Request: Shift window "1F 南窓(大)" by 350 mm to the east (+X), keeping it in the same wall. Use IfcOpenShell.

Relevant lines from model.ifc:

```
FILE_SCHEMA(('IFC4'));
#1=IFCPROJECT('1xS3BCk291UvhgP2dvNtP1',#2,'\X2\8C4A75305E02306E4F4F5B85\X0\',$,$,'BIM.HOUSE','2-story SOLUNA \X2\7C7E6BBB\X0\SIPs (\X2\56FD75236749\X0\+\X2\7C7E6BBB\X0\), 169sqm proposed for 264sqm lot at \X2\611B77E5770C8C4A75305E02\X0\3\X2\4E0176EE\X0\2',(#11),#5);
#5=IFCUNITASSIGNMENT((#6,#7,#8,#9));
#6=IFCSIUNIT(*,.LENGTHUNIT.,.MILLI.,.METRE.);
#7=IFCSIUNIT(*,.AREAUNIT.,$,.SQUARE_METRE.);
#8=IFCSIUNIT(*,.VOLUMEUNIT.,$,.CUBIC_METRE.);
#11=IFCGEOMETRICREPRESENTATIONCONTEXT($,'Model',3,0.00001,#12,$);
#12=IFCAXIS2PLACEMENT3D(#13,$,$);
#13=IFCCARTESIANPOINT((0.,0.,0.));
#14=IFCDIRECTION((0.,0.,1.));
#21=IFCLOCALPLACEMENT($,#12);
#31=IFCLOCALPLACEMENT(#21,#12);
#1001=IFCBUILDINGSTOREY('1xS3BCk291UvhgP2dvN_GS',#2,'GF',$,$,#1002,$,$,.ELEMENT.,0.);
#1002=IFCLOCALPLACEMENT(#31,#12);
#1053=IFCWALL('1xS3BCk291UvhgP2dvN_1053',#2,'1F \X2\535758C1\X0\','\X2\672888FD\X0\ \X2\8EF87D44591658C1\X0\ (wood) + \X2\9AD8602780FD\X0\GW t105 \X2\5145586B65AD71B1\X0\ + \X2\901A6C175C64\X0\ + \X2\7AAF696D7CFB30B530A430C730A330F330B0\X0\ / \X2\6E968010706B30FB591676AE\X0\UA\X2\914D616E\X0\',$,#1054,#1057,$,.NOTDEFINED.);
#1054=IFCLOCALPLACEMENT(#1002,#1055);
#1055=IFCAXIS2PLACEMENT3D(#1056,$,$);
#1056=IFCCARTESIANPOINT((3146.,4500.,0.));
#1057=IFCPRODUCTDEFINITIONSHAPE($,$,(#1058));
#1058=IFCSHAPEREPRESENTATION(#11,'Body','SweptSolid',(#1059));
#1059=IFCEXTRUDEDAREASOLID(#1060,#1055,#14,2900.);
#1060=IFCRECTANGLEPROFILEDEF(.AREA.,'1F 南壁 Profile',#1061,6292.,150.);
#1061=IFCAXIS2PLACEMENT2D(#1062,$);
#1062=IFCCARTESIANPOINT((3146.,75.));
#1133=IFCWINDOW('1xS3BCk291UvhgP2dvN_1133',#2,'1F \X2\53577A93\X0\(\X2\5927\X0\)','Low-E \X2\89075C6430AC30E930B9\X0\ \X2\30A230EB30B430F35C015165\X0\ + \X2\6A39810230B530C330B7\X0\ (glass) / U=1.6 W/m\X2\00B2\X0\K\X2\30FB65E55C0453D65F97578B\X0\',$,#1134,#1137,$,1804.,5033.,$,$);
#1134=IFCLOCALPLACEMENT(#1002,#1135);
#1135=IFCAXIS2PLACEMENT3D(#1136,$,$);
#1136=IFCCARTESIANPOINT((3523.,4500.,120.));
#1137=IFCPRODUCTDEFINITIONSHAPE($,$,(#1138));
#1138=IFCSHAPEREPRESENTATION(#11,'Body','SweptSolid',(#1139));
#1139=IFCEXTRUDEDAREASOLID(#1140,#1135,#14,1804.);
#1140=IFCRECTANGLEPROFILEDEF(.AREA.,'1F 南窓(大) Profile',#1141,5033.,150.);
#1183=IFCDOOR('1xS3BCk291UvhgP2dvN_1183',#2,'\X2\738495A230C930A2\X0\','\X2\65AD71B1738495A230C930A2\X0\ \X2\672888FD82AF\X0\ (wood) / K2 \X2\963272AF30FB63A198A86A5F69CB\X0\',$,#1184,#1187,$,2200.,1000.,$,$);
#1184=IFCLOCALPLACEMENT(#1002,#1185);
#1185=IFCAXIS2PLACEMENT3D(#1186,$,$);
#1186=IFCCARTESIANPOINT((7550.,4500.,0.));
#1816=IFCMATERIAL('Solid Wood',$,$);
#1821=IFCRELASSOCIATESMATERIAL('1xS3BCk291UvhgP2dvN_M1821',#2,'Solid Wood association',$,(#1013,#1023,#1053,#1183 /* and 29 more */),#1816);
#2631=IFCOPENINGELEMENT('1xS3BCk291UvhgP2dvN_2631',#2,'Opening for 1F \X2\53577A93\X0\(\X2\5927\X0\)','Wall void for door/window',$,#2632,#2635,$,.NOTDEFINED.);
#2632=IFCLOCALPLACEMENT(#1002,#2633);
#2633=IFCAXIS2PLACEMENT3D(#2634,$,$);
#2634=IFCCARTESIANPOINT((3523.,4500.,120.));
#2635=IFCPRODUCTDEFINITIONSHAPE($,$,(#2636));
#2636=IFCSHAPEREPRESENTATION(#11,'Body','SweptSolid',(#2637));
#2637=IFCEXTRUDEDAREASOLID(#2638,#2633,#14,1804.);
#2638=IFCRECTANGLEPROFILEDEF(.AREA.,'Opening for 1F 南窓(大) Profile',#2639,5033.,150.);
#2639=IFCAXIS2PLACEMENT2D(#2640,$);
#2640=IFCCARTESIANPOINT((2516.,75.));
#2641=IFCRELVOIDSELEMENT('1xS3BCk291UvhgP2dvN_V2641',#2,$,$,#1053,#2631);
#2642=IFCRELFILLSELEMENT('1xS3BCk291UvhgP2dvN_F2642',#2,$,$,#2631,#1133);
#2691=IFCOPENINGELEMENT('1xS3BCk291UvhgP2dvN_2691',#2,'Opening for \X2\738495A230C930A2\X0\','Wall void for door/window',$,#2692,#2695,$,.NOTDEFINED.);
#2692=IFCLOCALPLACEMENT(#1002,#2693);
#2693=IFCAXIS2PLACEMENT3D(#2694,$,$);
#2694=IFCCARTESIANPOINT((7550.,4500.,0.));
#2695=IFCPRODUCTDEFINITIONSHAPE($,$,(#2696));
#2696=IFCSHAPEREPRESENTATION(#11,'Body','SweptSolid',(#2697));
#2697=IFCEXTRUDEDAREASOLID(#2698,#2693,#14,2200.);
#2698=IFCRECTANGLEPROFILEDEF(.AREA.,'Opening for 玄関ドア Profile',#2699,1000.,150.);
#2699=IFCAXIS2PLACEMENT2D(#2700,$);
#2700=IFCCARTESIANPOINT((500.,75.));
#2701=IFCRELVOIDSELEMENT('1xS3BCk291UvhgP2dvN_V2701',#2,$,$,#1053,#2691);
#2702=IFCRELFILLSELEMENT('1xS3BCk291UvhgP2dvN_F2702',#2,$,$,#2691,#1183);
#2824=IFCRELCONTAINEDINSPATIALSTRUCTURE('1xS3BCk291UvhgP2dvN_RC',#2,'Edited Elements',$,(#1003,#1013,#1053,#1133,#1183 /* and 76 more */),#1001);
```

```python
import ifcopenshell
import ifcopenshell.api.geometry
import ifcopenshell.util.placement

model = ifcopenshell.open("model.ifc")

window = model.by_guid("1xS3BCk291UvhgP2dvN_1133")
opening = window.FillsVoids[0].RelatingOpeningElement
wall = opening.VoidsElements[0].RelatingBuildingElement

wall_matrix = ifcopenshell.util.placement.get_local_placement(wall.ObjectPlacement)
shift = wall_matrix[:3, 0] * 350.0
before = ifcopenshell.util.placement.get_local_placement(window.ObjectPlacement)[:3, 3].copy()

# The window is not placed relative to its opening, so move both.
for product in (opening, window):
    matrix = ifcopenshell.util.placement.get_local_placement(product.ObjectPlacement)
    matrix[:3, 3] += shift
    ifcopenshell.api.geometry.edit_object_placement(model, product=product, matrix=matrix, is_si=False)

after = ifcopenshell.util.placement.get_local_placement(window.ObjectPlacement)[:3, 3]
print("window moved by", (after - before).round(3) + 0.0)

model.write("model_edited.ifc")
```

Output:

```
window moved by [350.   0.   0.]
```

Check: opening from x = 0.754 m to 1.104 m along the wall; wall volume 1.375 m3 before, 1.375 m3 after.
